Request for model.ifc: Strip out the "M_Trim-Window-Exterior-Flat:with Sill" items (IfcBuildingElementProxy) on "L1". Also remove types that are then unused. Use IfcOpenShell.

First a look at what the model holds.

```python
import ifcopenshell
import ifcopenshell.util.element

model = ifcopenshell.open("model.ifc")
print(model.schema)
storey = next(s for s in model.by_type("IfcBuildingStorey") if s.Name == "L1")
proxies = [e for e in ifcopenshell.util.element.get_decomposition(storey) if e.is_a("IfcBuildingElementProxy")]
seen = {}
for e in proxies:
    element_type = ifcopenshell.util.element.get_type(e)
    name = element_type.Name if element_type not in (None, e) else None
    seen[name] = seen.get(name, 0) + 1
for name, count in sorted(seen.items(), key=str):
    print(count, "x", name)
```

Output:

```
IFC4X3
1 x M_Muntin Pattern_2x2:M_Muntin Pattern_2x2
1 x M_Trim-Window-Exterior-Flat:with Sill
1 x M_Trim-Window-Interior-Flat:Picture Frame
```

```python
import ifcopenshell
import ifcopenshell.api.root
import ifcopenshell.util.element

model = ifcopenshell.open("model.ifc")

storey = next(s for s in model.by_type("IfcBuildingStorey") if s.Name == "L1")
proxies = [e for e in ifcopenshell.util.element.get_decomposition(storey) if e.is_a("IfcBuildingElementProxy")]
targets = [e for e in proxies if (t := ifcopenshell.util.element.get_type(e)) not in (None, e) and t.Name == "M_Trim-Window-Exterior-Flat:with Sill"]
types = {ifcopenshell.util.element.get_type(e) for e in targets} - {None, *targets}

for e in targets:
    ifcopenshell.api.root.remove_product(model, product=e)
print(len(targets), "removed")

unused = [t for t in types if not ifcopenshell.util.element.get_types(t)]
for t in unused:
    ifcopenshell.api.root.remove_product(model, product=t)
print(len(unused), "unused types removed")

model.write("model_updated.ifc")
```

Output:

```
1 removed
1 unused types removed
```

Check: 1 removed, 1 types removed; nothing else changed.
